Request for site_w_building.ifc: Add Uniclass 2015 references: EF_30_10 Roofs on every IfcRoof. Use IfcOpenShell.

First a look at what the model holds.

```python
import ifcopenshell

model = ifcopenshell.open("site_w_building.ifc")
print(model.schema)
print("classifications:", [c.Name for c in model.by_type("IfcClassification")])
for ifc_class in ("IfcDoor", "IfcRoof", "IfcStair", "IfcWall", "IfcWindow"):
    print(ifc_class, len(model.by_type(ifc_class)))
```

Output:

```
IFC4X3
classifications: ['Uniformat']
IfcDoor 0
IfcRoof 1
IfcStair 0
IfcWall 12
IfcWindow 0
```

```python
import ifcopenshell
import ifcopenshell.api.classification

model = ifcopenshell.open("site_w_building.ifc")

system = ifcopenshell.api.classification.add_classification(model, classification="Uniclass 2015")

codes = {
    "IfcRoof": ("EF_30_10", "Roofs"),
}
for ifc_class, (code, name) in codes.items():
    products = model.by_type(ifc_class)
    ifcopenshell.api.classification.add_reference(
        model, products=products, classification=system, identification=code, name=name
    )
    print(code, len(products))

model.write("site_w_building_v2.ifc")
```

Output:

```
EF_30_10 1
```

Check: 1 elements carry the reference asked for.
